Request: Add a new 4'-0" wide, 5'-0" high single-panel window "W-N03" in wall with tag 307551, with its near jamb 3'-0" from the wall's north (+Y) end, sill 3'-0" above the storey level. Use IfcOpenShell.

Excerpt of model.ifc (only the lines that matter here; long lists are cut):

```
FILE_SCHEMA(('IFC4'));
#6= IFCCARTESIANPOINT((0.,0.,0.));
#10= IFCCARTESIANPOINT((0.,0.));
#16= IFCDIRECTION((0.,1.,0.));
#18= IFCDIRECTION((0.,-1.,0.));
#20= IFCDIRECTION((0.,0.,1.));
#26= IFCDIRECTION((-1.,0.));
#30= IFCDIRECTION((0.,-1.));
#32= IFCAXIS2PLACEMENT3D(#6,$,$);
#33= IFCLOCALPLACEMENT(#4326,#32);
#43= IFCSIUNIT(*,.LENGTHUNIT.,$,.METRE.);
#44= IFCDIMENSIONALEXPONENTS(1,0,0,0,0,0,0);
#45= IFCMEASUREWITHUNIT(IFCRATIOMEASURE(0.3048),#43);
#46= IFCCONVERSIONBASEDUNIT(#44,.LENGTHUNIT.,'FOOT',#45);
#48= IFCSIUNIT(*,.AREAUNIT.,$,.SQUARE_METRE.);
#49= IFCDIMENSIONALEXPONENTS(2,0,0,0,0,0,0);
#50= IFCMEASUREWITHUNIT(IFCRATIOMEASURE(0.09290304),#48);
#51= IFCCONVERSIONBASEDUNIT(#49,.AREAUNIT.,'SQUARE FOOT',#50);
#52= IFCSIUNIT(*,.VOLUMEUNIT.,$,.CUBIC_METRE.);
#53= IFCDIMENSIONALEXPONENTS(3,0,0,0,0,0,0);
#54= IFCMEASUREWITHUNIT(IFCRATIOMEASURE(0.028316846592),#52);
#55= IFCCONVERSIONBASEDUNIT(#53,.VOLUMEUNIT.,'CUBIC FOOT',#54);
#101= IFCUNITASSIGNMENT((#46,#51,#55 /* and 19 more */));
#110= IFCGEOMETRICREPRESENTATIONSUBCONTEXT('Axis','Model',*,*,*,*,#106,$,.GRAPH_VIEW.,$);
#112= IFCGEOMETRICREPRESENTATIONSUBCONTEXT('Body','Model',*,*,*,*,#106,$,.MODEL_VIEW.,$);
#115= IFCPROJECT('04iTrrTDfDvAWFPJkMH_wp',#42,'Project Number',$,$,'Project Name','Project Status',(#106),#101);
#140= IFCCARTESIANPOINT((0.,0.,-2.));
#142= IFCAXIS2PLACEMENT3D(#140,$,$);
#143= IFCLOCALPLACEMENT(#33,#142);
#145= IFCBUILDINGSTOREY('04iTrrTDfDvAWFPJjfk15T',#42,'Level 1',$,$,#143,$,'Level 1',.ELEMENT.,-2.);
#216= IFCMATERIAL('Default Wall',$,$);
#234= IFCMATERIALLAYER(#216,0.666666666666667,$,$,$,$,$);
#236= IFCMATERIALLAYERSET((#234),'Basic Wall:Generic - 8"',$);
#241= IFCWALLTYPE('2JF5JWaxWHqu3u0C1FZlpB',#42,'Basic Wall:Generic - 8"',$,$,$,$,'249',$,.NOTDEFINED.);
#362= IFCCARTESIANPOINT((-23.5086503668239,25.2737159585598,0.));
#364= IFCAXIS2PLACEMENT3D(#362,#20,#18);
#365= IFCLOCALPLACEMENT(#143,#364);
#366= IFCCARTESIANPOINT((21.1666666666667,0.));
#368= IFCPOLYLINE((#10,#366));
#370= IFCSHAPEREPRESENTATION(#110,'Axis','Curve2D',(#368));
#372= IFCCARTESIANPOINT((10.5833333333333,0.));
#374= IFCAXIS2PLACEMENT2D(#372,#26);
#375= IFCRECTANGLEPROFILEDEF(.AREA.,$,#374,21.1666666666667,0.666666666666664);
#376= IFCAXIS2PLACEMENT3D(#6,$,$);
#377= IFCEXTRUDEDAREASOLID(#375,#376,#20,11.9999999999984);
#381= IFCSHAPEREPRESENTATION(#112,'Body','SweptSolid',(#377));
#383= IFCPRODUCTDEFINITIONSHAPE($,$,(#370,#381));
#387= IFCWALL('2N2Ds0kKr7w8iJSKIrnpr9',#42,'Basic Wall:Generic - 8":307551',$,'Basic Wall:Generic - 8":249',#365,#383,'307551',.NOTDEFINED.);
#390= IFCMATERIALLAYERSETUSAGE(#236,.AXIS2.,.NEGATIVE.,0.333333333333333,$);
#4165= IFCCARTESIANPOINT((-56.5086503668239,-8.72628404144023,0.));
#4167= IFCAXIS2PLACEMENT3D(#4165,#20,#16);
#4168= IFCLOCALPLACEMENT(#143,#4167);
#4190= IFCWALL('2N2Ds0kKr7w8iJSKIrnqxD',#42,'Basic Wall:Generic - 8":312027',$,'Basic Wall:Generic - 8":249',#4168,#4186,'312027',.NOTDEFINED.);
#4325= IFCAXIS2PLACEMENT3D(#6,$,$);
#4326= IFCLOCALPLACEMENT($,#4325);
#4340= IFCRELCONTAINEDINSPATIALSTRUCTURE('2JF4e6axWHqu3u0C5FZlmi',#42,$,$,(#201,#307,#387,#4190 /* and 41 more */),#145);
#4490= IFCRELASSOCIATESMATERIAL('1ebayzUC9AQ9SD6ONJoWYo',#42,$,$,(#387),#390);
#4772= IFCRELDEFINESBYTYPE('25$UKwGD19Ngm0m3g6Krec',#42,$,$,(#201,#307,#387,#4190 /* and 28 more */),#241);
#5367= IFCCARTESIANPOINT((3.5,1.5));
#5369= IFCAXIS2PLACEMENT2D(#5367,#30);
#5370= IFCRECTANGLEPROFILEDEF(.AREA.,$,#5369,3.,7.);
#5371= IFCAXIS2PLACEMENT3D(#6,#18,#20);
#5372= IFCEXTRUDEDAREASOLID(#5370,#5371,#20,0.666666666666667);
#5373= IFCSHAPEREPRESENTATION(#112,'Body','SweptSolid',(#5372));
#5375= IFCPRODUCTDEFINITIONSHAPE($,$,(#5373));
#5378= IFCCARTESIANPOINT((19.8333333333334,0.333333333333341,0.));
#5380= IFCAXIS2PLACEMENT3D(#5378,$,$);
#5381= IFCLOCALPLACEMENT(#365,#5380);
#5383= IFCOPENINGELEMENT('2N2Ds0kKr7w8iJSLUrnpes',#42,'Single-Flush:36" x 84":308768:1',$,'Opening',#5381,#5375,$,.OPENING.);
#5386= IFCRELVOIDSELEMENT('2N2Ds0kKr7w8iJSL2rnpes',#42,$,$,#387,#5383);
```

```python
import numpy as np
import ifcopenshell
import ifcopenshell.api.feature
import ifcopenshell.api.geometry
import ifcopenshell.api.root
import ifcopenshell.api.spatial
import ifcopenshell.geom
import ifcopenshell.util.element
import ifcopenshell.util.placement
import ifcopenshell.util.representation
import ifcopenshell.util.shape
import ifcopenshell.util.unit

model = ifcopenshell.open("model.ifc")
unit_scale = ifcopenshell.util.unit.calculate_unit_scale(model)
settings = ifcopenshell.geom.settings()


def volume(element):
    """Net volume in cubic metres, openings subtracted."""
    shape = ifcopenshell.geom.create_shape(settings, element)
    return ifcopenshell.util.shape.get_volume(shape.geometry)


wall = model.by_guid("2N2Ds0kKr7w8iJSKIrnpr9")
storey = ifcopenshell.util.element.get_container(wall, ifc_class="IfcBuildingStorey")
context = ifcopenshell.util.representation.get_context(model, "Model", "Body", "MODEL_VIEW")
before = volume(wall)

width, height, from_end, sill = 1.2192, 1.524, 0.9144, 0.9144  # metres

# The wall runs along its own X axis, and the end named is its -X end.
wall_shape = ifcopenshell.geom.create_shape(settings, wall)
x, y, z = ifcopenshell.util.shape.get_vertices(wall_shape.geometry).T
start = x.min() + from_end
face, thickness = float(y.min()), float(y.max() - y.min())
wall_matrix = ifcopenshell.util.placement.get_local_placement(wall.ObjectPlacement)
level = ifcopenshell.util.placement.get_local_placement(storey.ObjectPlacement)[2, 3]


def in_wall(x, y):
    """Placement at x, y metres in the wall's axes, at sill height."""
    matrix = wall_matrix.copy()
    matrix[:, 3] = wall_matrix @ np.array([x / unit_scale, y / unit_scale, 0.0, 1.0])
    matrix[2, 3] = level + sill / unit_scale
    return matrix


# Opening: a box that overshoots both wall faces by 50 mm.
opening = ifcopenshell.api.root.create_entity(model, ifc_class="IfcOpeningElement", predefined_type="OPENING")
box = ifcopenshell.api.geometry.add_wall_representation(
    model, context=context, length=width, height=height, thickness=thickness + 0.1
)
ifcopenshell.api.geometry.assign_representation(model, product=opening, representation=box)
ifcopenshell.api.geometry.edit_object_placement(model, product=opening, matrix=in_wall(start, face - 0.05), is_si=False)
ifcopenshell.api.feature.add_feature(model, feature=opening, element=wall)

window = ifcopenshell.api.root.create_entity(model, ifc_class="IfcWindow", name="W-N03", predefined_type="WINDOW")
window.OverallWidth, window.OverallHeight = width / unit_scale, height / unit_scale
window.PartitioningType = "SINGLE_PANEL"
body = ifcopenshell.api.geometry.add_window_representation(
    model,
    context=context,
    overall_width=window.OverallWidth,
    overall_height=window.OverallHeight,
    partition_type="SINGLE_PANEL",
)
ifcopenshell.api.geometry.assign_representation(model, product=window, representation=body)
ifcopenshell.api.spatial.assign_container(model, products=[window], relating_structure=storey)
ifcopenshell.api.feature.add_filling(model, opening=opening, element=window)

# Centre the window in the wall's thickness.
ifcopenshell.api.geometry.edit_object_placement(model, product=window, matrix=in_wall(start, face), is_si=False)
window_shape = ifcopenshell.geom.create_shape(settings, window)
depth = ifcopenshell.util.shape.get_vertices(window_shape.geometry)[:, 1]
offset = face + thickness / 2 - (depth.min() + depth.max()) / 2
ifcopenshell.api.geometry.edit_object_placement(model, product=window, matrix=in_wall(start, offset), is_si=False)

after = volume(wall)

print(f"wall volume {before:.3f} -> {after:.3f} m3")

model.write("model-out.ifc")
```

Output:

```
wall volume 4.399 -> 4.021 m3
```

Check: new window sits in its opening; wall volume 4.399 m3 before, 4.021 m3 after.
